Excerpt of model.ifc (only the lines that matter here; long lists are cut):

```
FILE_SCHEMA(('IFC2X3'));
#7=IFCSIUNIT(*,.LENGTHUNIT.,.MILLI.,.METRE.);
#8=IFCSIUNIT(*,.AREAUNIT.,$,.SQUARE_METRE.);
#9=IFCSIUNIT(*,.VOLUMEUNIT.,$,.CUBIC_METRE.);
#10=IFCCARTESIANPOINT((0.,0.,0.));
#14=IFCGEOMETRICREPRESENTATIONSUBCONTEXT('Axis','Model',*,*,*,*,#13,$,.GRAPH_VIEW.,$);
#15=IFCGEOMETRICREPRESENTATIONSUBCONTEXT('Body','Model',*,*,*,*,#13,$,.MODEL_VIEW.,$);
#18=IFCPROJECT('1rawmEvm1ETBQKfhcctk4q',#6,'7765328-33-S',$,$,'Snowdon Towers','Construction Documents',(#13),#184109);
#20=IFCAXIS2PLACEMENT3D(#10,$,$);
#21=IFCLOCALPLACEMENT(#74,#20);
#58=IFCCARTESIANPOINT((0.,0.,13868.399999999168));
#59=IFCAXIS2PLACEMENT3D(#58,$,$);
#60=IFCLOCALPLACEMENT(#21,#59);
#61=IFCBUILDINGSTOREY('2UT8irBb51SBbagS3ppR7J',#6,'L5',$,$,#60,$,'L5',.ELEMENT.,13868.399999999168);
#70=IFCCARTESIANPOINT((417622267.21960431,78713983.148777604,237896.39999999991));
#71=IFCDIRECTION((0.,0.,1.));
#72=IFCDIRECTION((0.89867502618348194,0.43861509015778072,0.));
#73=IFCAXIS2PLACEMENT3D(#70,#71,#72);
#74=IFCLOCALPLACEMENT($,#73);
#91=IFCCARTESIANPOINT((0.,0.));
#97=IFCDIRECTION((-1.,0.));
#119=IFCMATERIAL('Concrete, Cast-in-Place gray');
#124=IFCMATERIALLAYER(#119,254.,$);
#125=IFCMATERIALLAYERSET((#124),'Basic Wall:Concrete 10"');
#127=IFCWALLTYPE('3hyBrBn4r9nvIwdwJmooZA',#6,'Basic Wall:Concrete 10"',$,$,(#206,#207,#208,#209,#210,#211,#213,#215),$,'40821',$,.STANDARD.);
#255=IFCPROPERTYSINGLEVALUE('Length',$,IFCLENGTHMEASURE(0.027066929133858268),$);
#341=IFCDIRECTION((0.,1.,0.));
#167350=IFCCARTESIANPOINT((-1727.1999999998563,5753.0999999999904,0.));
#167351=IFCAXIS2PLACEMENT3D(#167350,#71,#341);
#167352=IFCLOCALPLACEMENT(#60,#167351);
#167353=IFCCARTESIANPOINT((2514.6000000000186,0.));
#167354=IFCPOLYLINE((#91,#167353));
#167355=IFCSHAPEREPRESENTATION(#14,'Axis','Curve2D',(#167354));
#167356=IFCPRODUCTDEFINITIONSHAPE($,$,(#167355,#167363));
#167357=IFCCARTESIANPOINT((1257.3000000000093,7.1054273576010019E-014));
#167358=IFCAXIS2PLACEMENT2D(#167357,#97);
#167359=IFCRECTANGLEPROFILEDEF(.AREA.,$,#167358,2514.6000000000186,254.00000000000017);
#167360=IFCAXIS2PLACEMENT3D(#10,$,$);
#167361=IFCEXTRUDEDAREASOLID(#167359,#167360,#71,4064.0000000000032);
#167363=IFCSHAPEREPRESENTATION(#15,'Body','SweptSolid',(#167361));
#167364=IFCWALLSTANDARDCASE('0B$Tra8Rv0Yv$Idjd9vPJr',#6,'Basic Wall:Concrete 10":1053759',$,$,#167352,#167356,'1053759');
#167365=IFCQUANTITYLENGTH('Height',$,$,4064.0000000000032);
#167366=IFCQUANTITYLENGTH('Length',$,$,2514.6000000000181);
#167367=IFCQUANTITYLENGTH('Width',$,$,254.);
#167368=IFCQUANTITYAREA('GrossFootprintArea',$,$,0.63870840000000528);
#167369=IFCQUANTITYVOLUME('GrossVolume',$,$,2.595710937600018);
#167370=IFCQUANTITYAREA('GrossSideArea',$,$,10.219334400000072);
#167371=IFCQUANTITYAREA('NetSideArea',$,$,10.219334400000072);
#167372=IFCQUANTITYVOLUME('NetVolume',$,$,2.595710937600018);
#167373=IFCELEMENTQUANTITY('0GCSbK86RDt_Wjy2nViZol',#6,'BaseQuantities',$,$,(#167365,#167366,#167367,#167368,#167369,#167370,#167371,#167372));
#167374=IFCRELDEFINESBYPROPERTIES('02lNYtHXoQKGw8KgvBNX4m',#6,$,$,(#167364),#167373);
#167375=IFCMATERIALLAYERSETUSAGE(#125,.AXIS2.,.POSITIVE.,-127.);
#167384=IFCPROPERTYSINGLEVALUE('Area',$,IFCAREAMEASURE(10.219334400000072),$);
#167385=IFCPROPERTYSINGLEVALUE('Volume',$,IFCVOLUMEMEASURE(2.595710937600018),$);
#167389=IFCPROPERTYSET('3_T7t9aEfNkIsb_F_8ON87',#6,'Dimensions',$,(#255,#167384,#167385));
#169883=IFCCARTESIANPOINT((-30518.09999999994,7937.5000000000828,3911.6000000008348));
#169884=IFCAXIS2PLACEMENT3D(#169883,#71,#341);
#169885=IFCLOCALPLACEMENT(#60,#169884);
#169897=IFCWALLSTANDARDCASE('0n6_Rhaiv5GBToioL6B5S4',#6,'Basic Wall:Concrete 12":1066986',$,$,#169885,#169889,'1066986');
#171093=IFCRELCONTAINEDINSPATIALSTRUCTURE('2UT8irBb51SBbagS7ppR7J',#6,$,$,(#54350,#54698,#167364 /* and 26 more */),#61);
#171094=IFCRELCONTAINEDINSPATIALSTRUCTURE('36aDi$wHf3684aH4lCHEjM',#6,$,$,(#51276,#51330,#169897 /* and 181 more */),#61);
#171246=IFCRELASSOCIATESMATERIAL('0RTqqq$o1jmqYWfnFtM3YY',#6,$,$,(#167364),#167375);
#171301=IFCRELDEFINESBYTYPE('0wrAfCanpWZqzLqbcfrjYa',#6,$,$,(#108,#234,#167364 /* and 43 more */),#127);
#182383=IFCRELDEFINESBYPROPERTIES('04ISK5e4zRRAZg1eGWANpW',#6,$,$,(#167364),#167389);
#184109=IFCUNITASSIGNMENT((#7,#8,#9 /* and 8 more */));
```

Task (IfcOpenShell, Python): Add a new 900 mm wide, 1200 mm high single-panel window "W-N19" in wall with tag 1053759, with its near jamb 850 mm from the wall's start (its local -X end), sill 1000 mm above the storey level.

```python
import numpy as np
import ifcopenshell
import ifcopenshell.api.feature
import ifcopenshell.api.geometry
import ifcopenshell.api.pset
import ifcopenshell.api.root
import ifcopenshell.api.spatial
import ifcopenshell.api.type
import ifcopenshell.geom
import ifcopenshell.util.element
import ifcopenshell.util.placement
import ifcopenshell.util.representation
import ifcopenshell.util.shape
import ifcopenshell.util.unit

model = ifcopenshell.open("model.ifc")
unit_scale = ifcopenshell.util.unit.calculate_unit_scale(model)
area_scale = ifcopenshell.util.unit.calculate_unit_scale(model, "AREAUNIT")
volume_scale = ifcopenshell.util.unit.calculate_unit_scale(model, "VOLUMEUNIT")
settings = ifcopenshell.geom.settings()


def volume(element):
    """Net volume in cubic metres, openings subtracted."""
    shape = ifcopenshell.geom.create_shape(settings, element)
    return ifcopenshell.util.shape.get_volume(shape.geometry)


wall = model.by_guid("0B$Tra8Rv0Yv$Idjd9vPJr")
storey = ifcopenshell.util.element.get_container(wall, ifc_class="IfcBuildingStorey")
context = ifcopenshell.util.representation.get_context(model, "Model", "Body", "MODEL_VIEW")
before = volume(wall)

width, height, from_end, sill = 0.9, 1.2, 0.85, 1  # metres

# The wall runs along its own X axis, and the end named is its -X end.
wall_shape = ifcopenshell.geom.create_shape(settings, wall)
x, y, z = ifcopenshell.util.shape.get_vertices(wall_shape.geometry).T
start = x.min() + from_end
face, thickness = float(y.min()), float(y.max() - y.min())
wall_matrix = ifcopenshell.util.placement.get_local_placement(wall.ObjectPlacement)
level = ifcopenshell.util.placement.get_local_placement(storey.ObjectPlacement)[2, 3]


def in_wall(x, y):
    """Placement at x, y metres in the wall's axes, at sill height."""
    matrix = wall_matrix.copy()
    matrix[:, 3] = wall_matrix @ np.array([x / unit_scale, y / unit_scale, 0.0, 1.0])
    matrix[2, 3] = level + sill / unit_scale
    return matrix


# Opening: a box that overshoots both wall faces by 50 mm.
opening = ifcopenshell.api.root.create_entity(model, ifc_class="IfcOpeningElement")
box = ifcopenshell.api.geometry.add_wall_representation(
    model, context=context, length=width, height=height, thickness=thickness + 0.1
)
ifcopenshell.api.geometry.assign_representation(model, product=opening, representation=box)
ifcopenshell.api.geometry.edit_object_placement(model, product=opening, matrix=in_wall(start, face - 0.05), is_si=False)
ifcopenshell.api.feature.add_feature(model, feature=opening, element=wall)

window = ifcopenshell.api.root.create_entity(model, ifc_class="IfcWindow", name="W-N19")
window.OverallWidth, window.OverallHeight = width / unit_scale, height / unit_scale
body = ifcopenshell.api.geometry.add_window_representation(
    model,
    context=context,
    overall_width=window.OverallWidth,
    overall_height=window.OverallHeight,
    partition_type="SINGLE_PANEL",
)
ifcopenshell.api.geometry.assign_representation(model, product=window, representation=body)
ifcopenshell.api.spatial.assign_container(model, products=[window], relating_structure=storey)
fills = ifcopenshell.api.feature.add_filling(model, opening=opening, element=window)
fills.OwnerHistory = window.OwnerHistory  # required in IFC2X3

# IFC2X3 keeps the operation on the window style.
style = ifcopenshell.api.root.create_entity(model, ifc_class="IfcWindowStyle", name="W-N19")
style.OperationType, style.ConstructionType = "SINGLE_PANEL", "NOTDEFINED"
style.ParameterTakesPrecedence = style.Sizeable = False
ifcopenshell.api.type.assign_type(model, related_objects=[window], relating_type=style)

# Centre the window in the wall's thickness.
ifcopenshell.api.geometry.edit_object_placement(model, product=window, matrix=in_wall(start, face), is_si=False)
window_shape = ifcopenshell.geom.create_shape(settings, window)
depth = ifcopenshell.util.shape.get_vertices(window_shape.geometry)[:, 1]
offset = face + thickness / 2 - (depth.min() + depth.max()) / 2
ifcopenshell.api.geometry.edit_object_placement(model, product=window, matrix=in_wall(start, offset), is_si=False)

after = volume(wall)

# Update the wall's stored quantities.
qto = model.by_id(ifcopenshell.util.element.get_pset(wall, "BaseQuantities", should_inherit=False)["id"])
ifcopenshell.api.pset.edit_qto(model, qto=qto, properties={
    "NetSideArea": after / thickness / area_scale,
    "NetVolume": after / volume_scale,
})
pset = model.by_id(ifcopenshell.util.element.get_pset(wall, "Dimensions", should_inherit=False)["id"])
ifcopenshell.api.pset.edit_pset(model, pset=pset, properties={
    "Area": model.create_entity("IfcAreaMeasure", after / thickness / area_scale),
    "Volume": model.create_entity("IfcVolumeMeasure", after / volume_scale),
})

print(f"wall volume {before:.3f} -> {after:.3f} m3")

model.write("model_v2.ifc")
```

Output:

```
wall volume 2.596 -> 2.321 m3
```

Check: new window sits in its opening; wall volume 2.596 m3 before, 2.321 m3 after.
